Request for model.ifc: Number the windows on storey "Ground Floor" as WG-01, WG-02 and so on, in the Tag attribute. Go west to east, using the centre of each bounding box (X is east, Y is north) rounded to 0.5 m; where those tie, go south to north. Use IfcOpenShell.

First a look at what the model holds.

```python
import ifcopenshell
import ifcopenshell.util.element
import ifcopenshell.util.placement

model = ifcopenshell.open("model.ifc")
print(model.schema)
storey = next(s for s in model.by_type("IfcBuildingStorey") if s.Name == "Ground Floor")
windows = [e for e in ifcopenshell.util.element.get_decomposition(storey) if e.is_a("IfcWindow")]
for e in sorted(windows, key=lambda e: e.id()):
    origin = ifcopenshell.util.placement.get_local_placement(e.ObjectPlacement)[:3, 3]
    print(e.id(), e.Tag, e.Name, origin.round(2) + 0.0, sep=" | ")
```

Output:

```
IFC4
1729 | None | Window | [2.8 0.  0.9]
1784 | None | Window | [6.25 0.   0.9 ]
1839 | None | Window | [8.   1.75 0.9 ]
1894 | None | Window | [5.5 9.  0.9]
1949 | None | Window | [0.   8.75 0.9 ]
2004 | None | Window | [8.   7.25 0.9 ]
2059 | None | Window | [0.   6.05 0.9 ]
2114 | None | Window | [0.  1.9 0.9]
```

```python
import ifcopenshell
import ifcopenshell.geom
import ifcopenshell.util.element
import ifcopenshell.util.shape

model = ifcopenshell.open("model.ifc")
settings = ifcopenshell.geom.settings()
settings.set("use-world-coords", True)


def centre(element):
    shape = ifcopenshell.geom.create_shape(settings, element)
    return ifcopenshell.util.shape.get_bbox_centroid(shape.geometry)


storey = next(s for s in model.by_type("IfcBuildingStorey") if s.Name == "Ground Floor")
windows = [e for e in ifcopenshell.util.element.get_decomposition(storey) if e.is_a("IfcWindow")]

# Insertion points can sit at a corner or the storey origin, so sort by the geometry (in metres).
centres = {e: centre(e) for e in windows}
windows.sort(key=lambda e: (round(centres[e][0] / 0.5), centres[e][1]))

for i, e in enumerate(windows, start=1):
    number = f"WG-{i:02d}"
    e.Tag = number
    print(e.id(), number)

model.write("model_v2.ifc")
```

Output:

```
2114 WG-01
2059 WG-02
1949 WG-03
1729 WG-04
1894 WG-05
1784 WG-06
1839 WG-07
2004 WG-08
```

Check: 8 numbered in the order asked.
